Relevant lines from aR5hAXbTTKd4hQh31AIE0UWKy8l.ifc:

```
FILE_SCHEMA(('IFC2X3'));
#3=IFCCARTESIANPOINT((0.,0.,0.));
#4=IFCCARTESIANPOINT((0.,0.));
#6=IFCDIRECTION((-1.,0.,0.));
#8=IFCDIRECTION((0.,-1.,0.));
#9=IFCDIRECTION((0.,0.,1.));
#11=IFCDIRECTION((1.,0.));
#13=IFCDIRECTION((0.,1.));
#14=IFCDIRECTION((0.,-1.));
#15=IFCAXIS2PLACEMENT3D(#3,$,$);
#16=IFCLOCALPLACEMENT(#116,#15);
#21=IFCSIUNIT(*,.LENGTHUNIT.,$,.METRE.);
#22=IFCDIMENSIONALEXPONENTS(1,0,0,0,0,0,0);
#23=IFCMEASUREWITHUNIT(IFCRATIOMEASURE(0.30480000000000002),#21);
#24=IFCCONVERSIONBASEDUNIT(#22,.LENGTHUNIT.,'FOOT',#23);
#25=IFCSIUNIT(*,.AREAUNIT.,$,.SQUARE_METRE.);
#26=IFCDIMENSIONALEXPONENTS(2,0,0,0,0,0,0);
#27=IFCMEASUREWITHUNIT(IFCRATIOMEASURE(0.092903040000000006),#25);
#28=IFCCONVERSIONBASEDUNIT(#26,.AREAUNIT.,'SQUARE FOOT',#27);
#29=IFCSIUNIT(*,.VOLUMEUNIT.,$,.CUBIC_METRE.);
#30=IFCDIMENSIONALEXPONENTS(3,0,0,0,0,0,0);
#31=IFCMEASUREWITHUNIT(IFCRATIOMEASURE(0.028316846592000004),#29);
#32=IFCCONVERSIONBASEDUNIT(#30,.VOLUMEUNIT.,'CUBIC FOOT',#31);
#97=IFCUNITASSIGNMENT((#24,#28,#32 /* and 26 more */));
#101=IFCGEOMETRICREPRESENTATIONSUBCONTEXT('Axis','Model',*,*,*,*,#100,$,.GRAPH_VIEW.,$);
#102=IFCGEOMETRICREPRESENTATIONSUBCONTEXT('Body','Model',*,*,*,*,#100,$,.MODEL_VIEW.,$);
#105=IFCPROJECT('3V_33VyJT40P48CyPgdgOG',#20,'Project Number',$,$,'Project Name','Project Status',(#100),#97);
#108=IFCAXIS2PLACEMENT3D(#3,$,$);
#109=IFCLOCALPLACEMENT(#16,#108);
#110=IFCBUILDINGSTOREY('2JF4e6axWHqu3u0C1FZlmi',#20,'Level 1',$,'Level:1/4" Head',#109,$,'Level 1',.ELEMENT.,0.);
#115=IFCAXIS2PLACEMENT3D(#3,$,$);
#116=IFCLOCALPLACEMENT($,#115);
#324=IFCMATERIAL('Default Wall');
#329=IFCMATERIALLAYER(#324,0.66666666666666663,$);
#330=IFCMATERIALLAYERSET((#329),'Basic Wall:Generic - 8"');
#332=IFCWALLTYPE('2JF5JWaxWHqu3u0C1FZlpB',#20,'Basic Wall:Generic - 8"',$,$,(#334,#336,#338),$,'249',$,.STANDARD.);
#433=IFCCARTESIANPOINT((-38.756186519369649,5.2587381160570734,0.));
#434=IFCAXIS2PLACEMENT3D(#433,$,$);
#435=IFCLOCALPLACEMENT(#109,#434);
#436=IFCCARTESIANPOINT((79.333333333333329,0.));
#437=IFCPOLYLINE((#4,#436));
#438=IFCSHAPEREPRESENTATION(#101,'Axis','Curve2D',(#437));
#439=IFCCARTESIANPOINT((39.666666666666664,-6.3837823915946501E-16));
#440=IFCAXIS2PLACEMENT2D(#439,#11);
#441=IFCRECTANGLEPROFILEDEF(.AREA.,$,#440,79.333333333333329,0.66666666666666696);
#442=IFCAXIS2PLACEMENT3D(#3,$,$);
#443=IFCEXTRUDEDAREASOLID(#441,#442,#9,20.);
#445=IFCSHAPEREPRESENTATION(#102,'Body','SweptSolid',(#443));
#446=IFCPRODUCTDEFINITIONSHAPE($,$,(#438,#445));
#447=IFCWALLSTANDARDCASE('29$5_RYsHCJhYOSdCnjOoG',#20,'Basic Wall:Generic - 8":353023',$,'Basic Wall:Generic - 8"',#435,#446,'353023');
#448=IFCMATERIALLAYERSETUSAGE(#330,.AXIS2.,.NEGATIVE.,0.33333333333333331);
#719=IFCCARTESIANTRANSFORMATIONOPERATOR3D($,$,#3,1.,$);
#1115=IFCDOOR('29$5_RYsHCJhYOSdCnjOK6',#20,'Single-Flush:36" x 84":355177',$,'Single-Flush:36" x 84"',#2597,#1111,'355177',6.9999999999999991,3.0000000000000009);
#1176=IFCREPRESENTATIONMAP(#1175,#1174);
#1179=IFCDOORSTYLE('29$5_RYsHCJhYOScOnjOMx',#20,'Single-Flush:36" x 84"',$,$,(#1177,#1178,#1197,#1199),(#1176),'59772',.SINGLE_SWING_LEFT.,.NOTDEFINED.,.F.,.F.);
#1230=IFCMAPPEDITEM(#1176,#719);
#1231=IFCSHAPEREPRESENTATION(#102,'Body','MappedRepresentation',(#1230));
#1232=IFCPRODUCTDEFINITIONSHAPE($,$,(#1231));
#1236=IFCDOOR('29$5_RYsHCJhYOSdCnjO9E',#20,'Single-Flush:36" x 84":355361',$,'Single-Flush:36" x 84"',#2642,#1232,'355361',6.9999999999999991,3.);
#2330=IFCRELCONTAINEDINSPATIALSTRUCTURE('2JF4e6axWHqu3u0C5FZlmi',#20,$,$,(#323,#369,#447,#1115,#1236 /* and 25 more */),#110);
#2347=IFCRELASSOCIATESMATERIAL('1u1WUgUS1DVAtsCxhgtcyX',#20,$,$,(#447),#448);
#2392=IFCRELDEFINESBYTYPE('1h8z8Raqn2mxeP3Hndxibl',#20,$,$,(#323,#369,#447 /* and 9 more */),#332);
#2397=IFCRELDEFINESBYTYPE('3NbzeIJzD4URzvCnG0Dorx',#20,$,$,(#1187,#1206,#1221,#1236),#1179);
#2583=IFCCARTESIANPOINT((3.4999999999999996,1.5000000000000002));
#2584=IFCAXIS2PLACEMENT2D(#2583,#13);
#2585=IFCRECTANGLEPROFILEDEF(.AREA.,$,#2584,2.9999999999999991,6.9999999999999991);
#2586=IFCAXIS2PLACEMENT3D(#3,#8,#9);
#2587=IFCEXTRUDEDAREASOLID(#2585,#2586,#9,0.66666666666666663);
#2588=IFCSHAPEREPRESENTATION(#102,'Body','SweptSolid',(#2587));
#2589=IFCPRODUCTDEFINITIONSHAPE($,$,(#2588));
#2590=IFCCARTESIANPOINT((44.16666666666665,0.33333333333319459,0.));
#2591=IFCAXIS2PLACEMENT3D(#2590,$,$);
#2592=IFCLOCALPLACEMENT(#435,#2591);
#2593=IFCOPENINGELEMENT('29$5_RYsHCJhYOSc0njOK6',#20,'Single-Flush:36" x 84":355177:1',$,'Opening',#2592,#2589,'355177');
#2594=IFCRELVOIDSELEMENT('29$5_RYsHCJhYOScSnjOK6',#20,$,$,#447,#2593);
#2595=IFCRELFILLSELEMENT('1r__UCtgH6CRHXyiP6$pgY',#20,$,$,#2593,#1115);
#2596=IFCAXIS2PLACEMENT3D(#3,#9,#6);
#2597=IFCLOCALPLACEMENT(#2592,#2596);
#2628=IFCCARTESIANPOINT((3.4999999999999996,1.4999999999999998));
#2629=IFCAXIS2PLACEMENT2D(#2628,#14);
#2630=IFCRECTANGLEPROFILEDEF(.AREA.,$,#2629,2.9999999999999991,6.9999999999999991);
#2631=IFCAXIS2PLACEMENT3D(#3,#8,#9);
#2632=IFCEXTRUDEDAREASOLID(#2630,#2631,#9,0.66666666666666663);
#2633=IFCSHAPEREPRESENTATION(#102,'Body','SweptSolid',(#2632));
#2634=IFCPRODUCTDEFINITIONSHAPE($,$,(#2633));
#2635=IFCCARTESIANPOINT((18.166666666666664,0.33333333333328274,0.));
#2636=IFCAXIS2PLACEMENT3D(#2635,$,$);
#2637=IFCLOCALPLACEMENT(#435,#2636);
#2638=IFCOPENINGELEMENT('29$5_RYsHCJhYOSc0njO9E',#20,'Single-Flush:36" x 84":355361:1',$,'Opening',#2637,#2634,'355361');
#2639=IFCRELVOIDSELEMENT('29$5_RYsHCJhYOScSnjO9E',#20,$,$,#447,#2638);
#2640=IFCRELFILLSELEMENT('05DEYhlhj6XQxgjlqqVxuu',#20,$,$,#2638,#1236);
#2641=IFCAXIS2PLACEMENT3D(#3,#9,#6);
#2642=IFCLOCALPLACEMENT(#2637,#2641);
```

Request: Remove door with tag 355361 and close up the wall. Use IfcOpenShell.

```python
import ifcopenshell
import ifcopenshell.api.feature
import ifcopenshell.api.root
import ifcopenshell.geom
import ifcopenshell.util.shape

model = ifcopenshell.open("aR5hAXbTTKd4hQh31AIE0UWKy8l.ifc")
settings = ifcopenshell.geom.settings()


def volume(element):
    """Net volume in cubic metres, openings subtracted."""
    shape = ifcopenshell.geom.create_shape(settings, element)
    return ifcopenshell.util.shape.get_volume(shape.geometry)


door = model.by_guid("29$5_RYsHCJhYOSdCnjO9E")
opening = door.FillsVoids[0].RelatingOpeningElement
wall = opening.VoidsElements[0].RelatingBuildingElement
before = volume(wall)

ifcopenshell.api.root.remove_product(model, product=door)
ifcopenshell.api.feature.remove_feature(model, feature=opening)

after = volume(wall)

print(f"wall volume {before:.3f} -> {after:.3f} m3")

model.write("aR5hAXbTTKd4hQh31AIE0UWKy8l_rev.ifc")
```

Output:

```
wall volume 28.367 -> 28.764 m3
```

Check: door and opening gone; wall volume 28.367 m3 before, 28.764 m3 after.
